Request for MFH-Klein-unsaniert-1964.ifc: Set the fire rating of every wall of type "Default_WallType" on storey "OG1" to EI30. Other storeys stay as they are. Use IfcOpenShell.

First a look at what the model holds.

```python
import ifcopenshell
import ifcopenshell.util.element

model = ifcopenshell.open("MFH-Klein-unsaniert-1964.ifc")
print(model.schema)
storey = next(s for s in model.by_type("IfcBuildingStorey") if s.Name == "OG1")
walls = [e for e in ifcopenshell.util.element.get_decomposition(storey) if e.is_a("IfcWall")]
seen = {}
for e in walls:
    element_type = ifcopenshell.util.element.get_type(e)
    key = (element_type.Name if element_type != e and element_type else None, ifcopenshell.util.element.get_pset(e, "Pset_WallCommon", "FireRating"))
    seen[key] = seen.get(key, 0) + 1
for (name, value), count in sorted(seen.items(), key=str):
    print(count, "x", name, "|", value)
```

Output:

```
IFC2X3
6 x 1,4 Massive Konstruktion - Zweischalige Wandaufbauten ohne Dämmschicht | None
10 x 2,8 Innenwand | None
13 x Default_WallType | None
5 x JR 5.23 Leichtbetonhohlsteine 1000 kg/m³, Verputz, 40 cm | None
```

```python
import ifcopenshell
import ifcopenshell.api.pset
import ifcopenshell.util.element

model = ifcopenshell.open("MFH-Klein-unsaniert-1964.ifc")

storey = next(s for s in model.by_type("IfcBuildingStorey") if s.Name == "OG1")
walls = [e for e in ifcopenshell.util.element.get_decomposition(storey) if e.is_a("IfcWall")]

count = 0
for e in walls:
    element_type = ifcopenshell.util.element.get_type(e)
    if element_type in (None, e) or element_type.Name != "Default_WallType":
        continue
    # add_pset returns the element's existing set when there is one.
    pset = ifcopenshell.api.pset.add_pset(model, product=e, name="Pset_WallCommon")
    ifcopenshell.api.pset.edit_pset(model, pset=pset, properties={"FireRating": "EI30"})
    count += 1

print(count, "walls updated")

model.write("MFH-Klein-unsaniert-1964_v2.ifc")
```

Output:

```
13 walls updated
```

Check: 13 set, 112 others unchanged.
